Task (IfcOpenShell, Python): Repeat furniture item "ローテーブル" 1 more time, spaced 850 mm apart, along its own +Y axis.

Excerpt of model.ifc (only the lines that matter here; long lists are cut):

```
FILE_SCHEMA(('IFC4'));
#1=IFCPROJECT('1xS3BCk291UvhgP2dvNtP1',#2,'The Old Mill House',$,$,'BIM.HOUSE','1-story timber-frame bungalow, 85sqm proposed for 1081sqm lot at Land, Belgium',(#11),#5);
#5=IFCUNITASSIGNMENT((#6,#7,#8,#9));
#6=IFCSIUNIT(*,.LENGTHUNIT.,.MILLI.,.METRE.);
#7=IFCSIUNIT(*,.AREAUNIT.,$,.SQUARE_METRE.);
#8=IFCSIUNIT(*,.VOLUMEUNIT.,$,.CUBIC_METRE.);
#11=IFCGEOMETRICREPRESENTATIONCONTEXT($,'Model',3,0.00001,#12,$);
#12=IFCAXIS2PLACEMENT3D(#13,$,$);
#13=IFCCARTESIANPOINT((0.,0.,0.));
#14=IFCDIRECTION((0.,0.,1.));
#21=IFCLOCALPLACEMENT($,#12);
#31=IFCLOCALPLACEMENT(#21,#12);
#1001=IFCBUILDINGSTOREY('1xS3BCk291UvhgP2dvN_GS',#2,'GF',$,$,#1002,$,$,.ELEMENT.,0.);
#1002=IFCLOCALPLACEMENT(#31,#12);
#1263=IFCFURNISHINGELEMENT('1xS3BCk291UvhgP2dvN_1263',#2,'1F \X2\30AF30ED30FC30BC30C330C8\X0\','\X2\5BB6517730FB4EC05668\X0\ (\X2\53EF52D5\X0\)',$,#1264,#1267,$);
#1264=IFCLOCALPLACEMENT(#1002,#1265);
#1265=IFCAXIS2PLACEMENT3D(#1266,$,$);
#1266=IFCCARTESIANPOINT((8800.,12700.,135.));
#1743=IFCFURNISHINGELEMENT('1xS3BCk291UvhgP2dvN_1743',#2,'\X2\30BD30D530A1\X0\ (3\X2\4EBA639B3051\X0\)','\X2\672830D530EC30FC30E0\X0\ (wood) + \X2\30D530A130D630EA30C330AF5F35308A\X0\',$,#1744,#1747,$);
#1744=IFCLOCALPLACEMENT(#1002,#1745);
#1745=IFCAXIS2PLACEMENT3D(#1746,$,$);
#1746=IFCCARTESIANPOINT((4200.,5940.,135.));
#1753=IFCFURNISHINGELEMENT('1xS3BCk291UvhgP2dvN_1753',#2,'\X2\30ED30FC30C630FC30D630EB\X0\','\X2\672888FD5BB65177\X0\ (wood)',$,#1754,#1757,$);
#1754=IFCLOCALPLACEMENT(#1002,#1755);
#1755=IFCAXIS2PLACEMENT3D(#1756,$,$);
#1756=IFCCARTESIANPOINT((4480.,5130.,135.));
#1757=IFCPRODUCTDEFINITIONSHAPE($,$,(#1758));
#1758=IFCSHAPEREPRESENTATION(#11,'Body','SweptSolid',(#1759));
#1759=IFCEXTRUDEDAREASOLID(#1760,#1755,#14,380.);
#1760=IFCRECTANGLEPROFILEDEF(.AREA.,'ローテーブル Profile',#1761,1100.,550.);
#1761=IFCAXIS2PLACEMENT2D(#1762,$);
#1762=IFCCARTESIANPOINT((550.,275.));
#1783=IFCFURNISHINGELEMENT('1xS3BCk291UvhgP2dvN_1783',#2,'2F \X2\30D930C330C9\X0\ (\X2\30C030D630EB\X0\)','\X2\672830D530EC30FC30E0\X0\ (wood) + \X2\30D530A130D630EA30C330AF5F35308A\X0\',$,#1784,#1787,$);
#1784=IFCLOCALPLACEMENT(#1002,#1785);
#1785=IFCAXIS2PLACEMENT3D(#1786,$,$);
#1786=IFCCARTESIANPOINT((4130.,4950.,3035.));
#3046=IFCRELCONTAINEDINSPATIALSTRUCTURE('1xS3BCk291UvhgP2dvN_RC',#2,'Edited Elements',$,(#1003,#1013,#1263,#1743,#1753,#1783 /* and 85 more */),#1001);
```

```python
import ifcopenshell
import ifcopenshell.api.geometry
import ifcopenshell.api.root
import ifcopenshell.util.element
import ifcopenshell.util.placement
import ifcopenshell.util.unit

model = ifcopenshell.open("model.ifc")
unit_scale = ifcopenshell.util.unit.calculate_unit_scale(model)


def reuse_history(source, copy):
    """copy_class also copies each property set's owner history, people and application; keep the originals."""
    for rel in copy.IsDefinedBy:
        if rel.is_a("IfcRelDefinesByProperties") and (history := rel.RelatingPropertyDefinition.OwnerHistory):
            rel.RelatingPropertyDefinition.OwnerHistory = source.OwnerHistory
            ifcopenshell.util.element.remove_deep2(model, history)


source = model.by_guid("1xS3BCk291UvhgP2dvN_1753")
base = ifcopenshell.util.placement.get_local_placement(source.ObjectPlacement)
step = base[:3, 1] * 0.85 / unit_scale

for i in range(1, 2):
    copy = ifcopenshell.api.root.copy_class(model, product=source)
    copy.Representation = ifcopenshell.util.element.copy_deep(
        model, source.Representation, exclude=["IfcGeometricRepresentationContext", "IfcRepresentationMap"]
    )
    reuse_history(source, copy)
    matrix = base.copy()
    matrix[:3, 3] += i * step
    print("added at", matrix[:3, 3].round(3) + 0.0)
    ifcopenshell.api.geometry.edit_object_placement(model, product=copy, matrix=matrix, is_si=False)

model.write("model_v2.ifc")
```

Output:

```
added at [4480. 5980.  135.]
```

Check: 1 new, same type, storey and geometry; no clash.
